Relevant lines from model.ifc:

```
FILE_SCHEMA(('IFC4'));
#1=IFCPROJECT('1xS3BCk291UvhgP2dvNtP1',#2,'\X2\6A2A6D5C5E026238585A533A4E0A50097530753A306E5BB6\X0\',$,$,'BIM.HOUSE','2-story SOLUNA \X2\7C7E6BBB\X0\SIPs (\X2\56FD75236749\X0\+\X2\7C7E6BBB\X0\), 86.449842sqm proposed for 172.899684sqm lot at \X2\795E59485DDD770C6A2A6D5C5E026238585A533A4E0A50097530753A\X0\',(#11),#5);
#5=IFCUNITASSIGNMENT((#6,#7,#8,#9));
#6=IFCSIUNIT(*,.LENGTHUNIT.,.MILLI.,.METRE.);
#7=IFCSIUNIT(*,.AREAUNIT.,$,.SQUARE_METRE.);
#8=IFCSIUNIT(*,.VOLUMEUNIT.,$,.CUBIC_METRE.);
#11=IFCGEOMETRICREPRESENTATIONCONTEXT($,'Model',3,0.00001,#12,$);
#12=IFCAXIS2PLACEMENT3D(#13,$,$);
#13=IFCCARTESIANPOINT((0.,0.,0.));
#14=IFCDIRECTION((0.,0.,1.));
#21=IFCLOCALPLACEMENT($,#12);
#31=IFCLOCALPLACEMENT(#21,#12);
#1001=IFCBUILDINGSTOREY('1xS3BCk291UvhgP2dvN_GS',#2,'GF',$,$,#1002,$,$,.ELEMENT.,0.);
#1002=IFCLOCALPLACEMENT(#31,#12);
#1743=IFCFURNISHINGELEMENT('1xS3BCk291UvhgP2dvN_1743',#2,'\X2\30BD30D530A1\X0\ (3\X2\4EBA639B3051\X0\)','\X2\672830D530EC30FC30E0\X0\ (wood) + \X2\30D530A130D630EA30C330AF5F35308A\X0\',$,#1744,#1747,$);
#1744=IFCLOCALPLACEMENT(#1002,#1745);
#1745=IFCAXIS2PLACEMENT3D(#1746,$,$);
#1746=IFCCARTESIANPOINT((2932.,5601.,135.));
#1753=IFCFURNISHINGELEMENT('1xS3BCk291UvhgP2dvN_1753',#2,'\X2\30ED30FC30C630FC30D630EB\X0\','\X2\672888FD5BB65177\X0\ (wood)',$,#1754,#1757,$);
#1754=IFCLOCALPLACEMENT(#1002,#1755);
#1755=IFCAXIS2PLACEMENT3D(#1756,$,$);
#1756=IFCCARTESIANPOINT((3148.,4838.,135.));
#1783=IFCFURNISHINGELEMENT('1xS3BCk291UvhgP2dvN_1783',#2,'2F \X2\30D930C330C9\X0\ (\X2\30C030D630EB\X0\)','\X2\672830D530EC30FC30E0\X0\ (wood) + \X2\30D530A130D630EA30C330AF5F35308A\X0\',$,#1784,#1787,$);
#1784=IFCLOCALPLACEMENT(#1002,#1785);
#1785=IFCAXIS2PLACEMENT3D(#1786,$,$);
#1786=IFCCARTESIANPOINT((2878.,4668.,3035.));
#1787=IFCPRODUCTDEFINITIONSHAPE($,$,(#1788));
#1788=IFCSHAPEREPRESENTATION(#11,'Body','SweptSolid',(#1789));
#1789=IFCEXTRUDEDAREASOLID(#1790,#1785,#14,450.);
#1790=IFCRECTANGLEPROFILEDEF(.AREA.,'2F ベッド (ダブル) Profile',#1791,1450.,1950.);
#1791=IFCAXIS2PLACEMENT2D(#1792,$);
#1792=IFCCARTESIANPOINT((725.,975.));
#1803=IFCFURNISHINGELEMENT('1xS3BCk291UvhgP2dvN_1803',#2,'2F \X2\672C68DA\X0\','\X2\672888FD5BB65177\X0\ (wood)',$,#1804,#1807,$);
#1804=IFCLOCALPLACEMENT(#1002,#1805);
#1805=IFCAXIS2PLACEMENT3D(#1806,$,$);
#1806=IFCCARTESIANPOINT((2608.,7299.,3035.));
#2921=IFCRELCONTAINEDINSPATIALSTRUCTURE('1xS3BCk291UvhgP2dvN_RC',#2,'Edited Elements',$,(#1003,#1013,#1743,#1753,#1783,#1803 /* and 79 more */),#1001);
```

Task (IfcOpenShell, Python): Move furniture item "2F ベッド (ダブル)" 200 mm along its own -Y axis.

```python
import ifcopenshell
import ifcopenshell.api.geometry
import ifcopenshell.util.placement
import ifcopenshell.util.unit

model = ifcopenshell.open("model.ifc")
unit_scale = ifcopenshell.util.unit.calculate_unit_scale(model)

item = model.by_guid("1xS3BCk291UvhgP2dvN_1783")
matrix = ifcopenshell.util.placement.get_local_placement(item.ObjectPlacement)
matrix[:3, 3] -= matrix[:3, 1] * 0.2 / unit_scale
ifcopenshell.api.geometry.edit_object_placement(model, product=item, matrix=matrix, is_si=False)

print(ifcopenshell.util.placement.get_local_placement(item.ObjectPlacement).round(3) + 0.0)

model.write("model_edited.ifc")
```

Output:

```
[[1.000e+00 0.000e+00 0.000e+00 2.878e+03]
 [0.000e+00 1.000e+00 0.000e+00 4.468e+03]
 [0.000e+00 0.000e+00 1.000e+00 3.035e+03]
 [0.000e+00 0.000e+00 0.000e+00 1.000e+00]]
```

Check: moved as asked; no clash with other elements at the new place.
